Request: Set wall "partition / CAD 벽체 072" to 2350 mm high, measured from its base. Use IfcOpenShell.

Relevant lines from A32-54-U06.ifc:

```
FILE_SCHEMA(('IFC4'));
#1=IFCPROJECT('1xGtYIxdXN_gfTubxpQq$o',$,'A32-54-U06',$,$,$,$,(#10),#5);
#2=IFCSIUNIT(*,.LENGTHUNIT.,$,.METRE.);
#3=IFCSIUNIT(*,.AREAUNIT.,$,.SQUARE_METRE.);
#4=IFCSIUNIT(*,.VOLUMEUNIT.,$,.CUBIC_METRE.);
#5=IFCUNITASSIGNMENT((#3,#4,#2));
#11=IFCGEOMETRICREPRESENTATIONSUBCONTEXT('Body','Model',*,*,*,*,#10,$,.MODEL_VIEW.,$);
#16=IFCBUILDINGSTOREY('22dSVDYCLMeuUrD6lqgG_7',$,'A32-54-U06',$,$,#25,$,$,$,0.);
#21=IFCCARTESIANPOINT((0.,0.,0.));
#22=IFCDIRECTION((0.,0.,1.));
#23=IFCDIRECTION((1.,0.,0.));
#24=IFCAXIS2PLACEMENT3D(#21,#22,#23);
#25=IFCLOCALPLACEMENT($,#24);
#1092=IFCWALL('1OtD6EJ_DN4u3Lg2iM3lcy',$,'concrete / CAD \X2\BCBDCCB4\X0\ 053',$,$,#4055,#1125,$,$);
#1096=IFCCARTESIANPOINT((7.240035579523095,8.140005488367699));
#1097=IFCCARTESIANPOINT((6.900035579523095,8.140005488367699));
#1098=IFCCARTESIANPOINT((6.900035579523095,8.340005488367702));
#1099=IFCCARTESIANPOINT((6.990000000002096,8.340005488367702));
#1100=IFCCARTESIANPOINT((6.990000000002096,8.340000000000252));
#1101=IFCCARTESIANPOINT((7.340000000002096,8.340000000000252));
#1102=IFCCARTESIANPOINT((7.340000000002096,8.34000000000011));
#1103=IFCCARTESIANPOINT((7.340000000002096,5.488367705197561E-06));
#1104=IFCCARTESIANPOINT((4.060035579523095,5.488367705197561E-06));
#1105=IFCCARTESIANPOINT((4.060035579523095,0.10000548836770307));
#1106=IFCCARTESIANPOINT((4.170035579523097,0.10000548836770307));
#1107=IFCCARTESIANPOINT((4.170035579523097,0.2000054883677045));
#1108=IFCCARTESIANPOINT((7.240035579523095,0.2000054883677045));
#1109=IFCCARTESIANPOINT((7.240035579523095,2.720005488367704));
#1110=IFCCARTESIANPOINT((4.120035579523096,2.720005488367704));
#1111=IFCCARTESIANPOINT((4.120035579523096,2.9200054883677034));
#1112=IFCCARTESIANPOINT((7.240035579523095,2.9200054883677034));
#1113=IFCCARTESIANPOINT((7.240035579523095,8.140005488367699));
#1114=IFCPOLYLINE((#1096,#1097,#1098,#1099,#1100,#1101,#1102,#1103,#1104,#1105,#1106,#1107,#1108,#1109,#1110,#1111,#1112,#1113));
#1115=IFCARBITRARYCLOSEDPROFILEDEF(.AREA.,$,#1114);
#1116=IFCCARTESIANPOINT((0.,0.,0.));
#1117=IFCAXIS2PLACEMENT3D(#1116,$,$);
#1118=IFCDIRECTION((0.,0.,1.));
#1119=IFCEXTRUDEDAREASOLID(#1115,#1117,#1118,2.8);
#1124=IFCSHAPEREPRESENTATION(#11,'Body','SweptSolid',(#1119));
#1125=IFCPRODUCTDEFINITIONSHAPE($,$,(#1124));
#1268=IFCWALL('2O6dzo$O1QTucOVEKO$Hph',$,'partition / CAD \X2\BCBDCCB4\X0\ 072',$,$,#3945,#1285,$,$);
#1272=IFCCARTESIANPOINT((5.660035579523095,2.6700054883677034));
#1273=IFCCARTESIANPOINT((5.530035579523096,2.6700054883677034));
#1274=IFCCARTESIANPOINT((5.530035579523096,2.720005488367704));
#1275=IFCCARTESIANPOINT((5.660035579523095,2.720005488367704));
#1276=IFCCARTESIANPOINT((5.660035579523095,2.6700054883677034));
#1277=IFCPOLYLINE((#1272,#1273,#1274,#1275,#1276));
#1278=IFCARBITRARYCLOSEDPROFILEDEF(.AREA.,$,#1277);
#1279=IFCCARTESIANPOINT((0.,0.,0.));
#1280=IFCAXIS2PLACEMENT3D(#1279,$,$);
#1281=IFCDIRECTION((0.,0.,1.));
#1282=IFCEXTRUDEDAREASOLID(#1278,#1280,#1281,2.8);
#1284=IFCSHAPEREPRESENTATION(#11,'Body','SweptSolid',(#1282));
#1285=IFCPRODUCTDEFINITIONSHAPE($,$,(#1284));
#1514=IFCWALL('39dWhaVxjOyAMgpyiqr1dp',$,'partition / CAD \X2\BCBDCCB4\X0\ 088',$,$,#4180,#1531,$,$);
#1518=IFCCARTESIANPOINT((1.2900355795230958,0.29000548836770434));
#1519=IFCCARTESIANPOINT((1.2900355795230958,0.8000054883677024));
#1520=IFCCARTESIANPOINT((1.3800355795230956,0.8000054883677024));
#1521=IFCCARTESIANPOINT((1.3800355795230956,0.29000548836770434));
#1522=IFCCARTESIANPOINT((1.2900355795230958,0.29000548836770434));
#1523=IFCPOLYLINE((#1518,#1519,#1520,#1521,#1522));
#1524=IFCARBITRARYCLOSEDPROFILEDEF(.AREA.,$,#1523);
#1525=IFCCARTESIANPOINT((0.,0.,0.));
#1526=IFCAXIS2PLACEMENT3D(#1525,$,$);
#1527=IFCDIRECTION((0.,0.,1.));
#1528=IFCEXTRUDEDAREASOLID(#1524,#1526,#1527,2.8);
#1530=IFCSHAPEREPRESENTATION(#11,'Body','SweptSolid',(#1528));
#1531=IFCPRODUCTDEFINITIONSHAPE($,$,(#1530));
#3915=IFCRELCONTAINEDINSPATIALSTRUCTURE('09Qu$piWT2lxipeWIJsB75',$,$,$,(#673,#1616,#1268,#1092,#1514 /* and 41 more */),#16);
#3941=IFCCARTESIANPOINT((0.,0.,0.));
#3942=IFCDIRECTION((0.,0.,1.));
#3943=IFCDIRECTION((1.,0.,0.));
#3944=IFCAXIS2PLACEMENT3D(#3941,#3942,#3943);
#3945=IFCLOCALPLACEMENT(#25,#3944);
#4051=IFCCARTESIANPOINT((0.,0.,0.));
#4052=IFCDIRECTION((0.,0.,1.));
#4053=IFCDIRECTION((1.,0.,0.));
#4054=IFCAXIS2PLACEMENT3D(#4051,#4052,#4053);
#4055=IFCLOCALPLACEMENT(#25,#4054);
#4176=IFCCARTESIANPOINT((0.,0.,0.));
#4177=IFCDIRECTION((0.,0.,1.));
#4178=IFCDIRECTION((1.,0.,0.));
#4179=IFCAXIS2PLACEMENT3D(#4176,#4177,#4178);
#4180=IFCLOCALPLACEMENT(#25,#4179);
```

```python
import ifcopenshell
import ifcopenshell.geom
import ifcopenshell.util.representation
import ifcopenshell.util.shape
import ifcopenshell.util.unit

model = ifcopenshell.open("A32-54-U06.ifc")
unit_scale = ifcopenshell.util.unit.calculate_unit_scale(model)
settings = ifcopenshell.geom.settings()


def volume(element):
    """Net volume in cubic metres, openings subtracted."""
    shape = ifcopenshell.geom.create_shape(settings, element)
    return ifcopenshell.util.shape.get_volume(shape.geometry)


wall = model.by_guid("2O6dzo$O1QTucOVEKO$Hph")
before = volume(wall)

body = ifcopenshell.util.representation.get_representation(wall, "Model", "Body")
solid = body.Items[0]
old_height = solid.Depth
solid.Depth = 2.35 / unit_scale
after = volume(wall)

print(f"height {old_height:g} -> {solid.Depth:g}, volume {before:.3f} -> {after:.3f} m3")

model.write("A32-54-U06_v2.ifc")
```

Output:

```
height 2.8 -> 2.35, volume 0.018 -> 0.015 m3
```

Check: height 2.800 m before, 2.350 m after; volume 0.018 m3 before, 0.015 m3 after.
